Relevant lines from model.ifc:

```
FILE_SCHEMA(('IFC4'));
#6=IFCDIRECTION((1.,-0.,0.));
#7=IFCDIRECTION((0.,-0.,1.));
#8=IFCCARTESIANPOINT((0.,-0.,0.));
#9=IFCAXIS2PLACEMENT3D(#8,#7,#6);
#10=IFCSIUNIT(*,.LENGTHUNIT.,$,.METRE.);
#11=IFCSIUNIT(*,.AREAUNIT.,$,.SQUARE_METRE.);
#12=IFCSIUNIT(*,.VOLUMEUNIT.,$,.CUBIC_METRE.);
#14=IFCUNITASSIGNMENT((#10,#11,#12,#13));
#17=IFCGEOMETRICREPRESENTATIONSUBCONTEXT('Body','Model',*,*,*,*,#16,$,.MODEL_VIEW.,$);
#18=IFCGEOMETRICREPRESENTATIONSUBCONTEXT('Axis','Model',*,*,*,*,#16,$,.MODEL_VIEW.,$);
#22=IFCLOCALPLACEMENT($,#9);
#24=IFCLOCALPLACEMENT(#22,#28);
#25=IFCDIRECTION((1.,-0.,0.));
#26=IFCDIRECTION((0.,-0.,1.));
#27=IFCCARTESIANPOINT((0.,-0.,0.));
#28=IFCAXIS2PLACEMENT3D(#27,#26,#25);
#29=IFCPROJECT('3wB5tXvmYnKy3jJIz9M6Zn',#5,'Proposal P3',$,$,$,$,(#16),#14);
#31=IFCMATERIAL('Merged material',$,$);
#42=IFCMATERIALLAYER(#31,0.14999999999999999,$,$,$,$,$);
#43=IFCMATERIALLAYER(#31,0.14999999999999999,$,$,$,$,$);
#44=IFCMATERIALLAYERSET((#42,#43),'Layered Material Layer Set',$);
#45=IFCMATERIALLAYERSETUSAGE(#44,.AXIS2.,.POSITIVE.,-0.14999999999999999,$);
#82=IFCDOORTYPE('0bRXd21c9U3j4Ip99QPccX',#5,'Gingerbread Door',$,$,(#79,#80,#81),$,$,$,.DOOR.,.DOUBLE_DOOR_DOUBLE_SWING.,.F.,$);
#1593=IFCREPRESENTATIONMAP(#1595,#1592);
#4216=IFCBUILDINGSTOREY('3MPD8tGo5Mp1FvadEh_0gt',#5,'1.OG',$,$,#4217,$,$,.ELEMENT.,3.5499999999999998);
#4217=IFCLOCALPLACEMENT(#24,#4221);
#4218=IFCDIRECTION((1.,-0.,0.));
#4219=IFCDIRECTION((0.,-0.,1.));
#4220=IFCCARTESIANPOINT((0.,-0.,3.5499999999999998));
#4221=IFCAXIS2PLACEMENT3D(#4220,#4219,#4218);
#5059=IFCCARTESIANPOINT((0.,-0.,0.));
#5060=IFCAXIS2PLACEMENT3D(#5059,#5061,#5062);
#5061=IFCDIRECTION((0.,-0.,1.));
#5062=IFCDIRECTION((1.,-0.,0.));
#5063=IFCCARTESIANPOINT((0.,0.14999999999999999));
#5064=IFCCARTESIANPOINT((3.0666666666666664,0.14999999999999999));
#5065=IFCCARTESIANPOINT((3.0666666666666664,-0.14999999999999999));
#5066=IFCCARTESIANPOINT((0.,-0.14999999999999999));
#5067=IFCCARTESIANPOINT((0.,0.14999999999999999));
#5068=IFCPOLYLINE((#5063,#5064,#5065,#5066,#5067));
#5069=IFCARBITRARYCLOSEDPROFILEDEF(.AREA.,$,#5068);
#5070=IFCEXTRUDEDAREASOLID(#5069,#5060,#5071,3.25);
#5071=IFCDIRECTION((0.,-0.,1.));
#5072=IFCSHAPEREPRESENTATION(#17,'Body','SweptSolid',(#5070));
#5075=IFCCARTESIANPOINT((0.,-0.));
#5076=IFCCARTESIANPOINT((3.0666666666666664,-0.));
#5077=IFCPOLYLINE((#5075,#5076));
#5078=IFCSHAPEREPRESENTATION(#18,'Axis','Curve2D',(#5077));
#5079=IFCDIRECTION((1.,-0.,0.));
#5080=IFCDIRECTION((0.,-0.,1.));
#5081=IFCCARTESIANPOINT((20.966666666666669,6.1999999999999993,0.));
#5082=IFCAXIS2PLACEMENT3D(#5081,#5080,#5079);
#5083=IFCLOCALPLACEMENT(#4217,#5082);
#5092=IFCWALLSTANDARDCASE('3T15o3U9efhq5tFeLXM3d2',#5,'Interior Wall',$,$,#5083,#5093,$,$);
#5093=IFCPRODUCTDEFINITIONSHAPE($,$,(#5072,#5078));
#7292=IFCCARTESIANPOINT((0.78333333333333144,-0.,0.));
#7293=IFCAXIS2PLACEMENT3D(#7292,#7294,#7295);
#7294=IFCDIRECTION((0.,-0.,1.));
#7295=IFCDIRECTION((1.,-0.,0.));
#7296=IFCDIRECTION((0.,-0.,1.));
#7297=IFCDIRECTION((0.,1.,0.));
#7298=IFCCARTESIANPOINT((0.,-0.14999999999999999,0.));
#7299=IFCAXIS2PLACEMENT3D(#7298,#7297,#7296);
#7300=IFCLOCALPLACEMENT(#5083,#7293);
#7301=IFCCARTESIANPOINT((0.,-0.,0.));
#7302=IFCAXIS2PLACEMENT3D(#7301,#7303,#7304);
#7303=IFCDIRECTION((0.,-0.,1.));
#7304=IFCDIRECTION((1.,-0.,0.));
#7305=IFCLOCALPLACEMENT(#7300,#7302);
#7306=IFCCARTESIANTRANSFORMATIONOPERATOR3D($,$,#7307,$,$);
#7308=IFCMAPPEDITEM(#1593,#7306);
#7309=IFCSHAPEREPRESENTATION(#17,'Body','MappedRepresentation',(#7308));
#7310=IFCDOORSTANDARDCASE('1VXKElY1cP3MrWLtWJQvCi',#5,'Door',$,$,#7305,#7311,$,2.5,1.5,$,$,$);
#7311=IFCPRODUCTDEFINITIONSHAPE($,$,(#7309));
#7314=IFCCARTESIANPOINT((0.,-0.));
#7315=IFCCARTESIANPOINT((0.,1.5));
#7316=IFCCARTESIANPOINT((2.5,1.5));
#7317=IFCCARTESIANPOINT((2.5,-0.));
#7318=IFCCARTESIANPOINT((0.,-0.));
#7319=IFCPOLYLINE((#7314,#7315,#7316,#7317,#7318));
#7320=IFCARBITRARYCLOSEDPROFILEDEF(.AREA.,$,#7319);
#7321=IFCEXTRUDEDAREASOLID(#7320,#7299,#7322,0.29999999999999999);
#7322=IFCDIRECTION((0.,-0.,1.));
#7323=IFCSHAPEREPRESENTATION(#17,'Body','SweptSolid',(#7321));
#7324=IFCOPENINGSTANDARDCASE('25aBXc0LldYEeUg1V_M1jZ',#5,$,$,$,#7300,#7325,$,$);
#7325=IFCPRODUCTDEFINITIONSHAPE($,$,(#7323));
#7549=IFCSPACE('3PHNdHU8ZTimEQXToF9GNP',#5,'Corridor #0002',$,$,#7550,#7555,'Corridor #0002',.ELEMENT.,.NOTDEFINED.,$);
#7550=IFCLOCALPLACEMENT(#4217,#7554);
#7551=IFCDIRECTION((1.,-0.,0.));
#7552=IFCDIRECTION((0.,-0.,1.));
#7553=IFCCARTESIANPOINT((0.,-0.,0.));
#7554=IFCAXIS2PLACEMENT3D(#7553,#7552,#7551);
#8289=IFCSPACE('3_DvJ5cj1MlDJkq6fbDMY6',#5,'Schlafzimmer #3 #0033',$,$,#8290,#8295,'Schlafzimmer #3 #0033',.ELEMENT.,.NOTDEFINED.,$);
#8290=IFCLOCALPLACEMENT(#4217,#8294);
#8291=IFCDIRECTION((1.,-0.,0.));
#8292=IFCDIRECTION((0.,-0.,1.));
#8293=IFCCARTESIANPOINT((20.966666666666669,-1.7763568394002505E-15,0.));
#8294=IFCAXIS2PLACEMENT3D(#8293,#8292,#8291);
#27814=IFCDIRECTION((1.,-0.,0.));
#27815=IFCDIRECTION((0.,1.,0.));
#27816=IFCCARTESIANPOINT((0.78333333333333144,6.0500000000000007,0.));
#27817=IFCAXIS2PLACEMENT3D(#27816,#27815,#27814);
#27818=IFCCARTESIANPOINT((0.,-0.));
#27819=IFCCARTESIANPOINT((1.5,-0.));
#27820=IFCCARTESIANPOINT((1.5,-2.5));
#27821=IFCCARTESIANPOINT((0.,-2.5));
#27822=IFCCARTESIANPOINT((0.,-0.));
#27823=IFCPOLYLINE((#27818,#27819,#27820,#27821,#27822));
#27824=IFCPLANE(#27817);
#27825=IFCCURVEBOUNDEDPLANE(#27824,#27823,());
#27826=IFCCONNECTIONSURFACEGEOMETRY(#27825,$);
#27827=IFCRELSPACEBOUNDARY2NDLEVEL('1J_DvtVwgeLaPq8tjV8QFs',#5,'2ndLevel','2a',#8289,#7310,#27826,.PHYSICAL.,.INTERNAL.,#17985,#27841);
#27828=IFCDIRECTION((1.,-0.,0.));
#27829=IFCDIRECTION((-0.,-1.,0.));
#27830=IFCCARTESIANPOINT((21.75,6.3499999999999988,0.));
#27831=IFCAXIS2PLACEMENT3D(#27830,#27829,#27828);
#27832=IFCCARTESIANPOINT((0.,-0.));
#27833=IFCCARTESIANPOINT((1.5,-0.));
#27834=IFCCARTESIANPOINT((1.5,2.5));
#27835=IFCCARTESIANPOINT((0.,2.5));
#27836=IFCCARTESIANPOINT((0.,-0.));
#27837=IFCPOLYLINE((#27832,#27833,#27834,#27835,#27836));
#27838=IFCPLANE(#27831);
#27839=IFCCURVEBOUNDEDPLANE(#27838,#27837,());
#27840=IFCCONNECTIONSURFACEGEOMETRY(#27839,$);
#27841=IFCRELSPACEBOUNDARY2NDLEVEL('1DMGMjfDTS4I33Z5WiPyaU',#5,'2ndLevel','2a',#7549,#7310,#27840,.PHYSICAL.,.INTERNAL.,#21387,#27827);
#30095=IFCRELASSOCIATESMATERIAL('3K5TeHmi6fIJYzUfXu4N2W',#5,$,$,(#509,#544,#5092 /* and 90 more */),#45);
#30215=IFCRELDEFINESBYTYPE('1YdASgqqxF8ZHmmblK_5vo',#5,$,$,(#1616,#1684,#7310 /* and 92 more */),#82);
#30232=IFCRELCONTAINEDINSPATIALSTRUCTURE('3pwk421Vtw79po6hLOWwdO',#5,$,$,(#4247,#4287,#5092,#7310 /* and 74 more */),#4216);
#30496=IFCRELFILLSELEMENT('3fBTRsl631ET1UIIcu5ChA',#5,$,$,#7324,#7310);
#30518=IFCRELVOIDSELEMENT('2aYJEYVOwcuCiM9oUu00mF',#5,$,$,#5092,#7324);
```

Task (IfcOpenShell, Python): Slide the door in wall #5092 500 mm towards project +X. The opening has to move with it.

```python
import numpy as np
import ifcopenshell
import ifcopenshell.api.geometry
import ifcopenshell.util.placement

model = ifcopenshell.open("model.ifc")

door = model.by_guid("1VXKElY1cP3MrWLtWJQvCi")
opening = door.FillsVoids[0].RelatingOpeningElement
wall = opening.VoidsElements[0].RelatingBuildingElement

wall_matrix = ifcopenshell.util.placement.get_local_placement(wall.ObjectPlacement)
shift = wall_matrix[:3, 0] * 0.5
before = ifcopenshell.util.placement.get_local_placement(door.ObjectPlacement)[:3, 3].copy()

# The door is placed relative to its opening, so it follows when the opening moves.
matrix = ifcopenshell.util.placement.get_local_placement(opening.ObjectPlacement)
matrix[:3, 3] += shift
ifcopenshell.api.geometry.edit_object_placement(
    model, product=opening, matrix=matrix, is_si=False, should_transform_children=True
)

# Space boundary surfaces are stored in each space's coordinates; move them too.
for rel in door.ProvidesBoundaries:
    if not rel.ConnectionGeometry:
        continue
    surface = rel.ConnectionGeometry.SurfaceOnRelatingElement.BasisSurface
    space_matrix = ifcopenshell.util.placement.get_local_placement(rel.RelatingSpace.ObjectPlacement)
    point = np.array(surface.Position.Location.Coordinates) + space_matrix[:3, :3].T @ shift
    surface.Position = model.createIfcAxis2Placement3D(
        model.createIfcCartesianPoint(point.tolist()), surface.Position.Axis, surface.Position.RefDirection
    )

after = ifcopenshell.util.placement.get_local_placement(door.ObjectPlacement)[:3, 3]
print("door moved by", (after - before).round(3) + 0.0)

model.write("model_updated.ifc")
```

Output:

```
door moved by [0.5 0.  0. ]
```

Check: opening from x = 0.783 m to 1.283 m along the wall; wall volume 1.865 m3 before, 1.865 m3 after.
